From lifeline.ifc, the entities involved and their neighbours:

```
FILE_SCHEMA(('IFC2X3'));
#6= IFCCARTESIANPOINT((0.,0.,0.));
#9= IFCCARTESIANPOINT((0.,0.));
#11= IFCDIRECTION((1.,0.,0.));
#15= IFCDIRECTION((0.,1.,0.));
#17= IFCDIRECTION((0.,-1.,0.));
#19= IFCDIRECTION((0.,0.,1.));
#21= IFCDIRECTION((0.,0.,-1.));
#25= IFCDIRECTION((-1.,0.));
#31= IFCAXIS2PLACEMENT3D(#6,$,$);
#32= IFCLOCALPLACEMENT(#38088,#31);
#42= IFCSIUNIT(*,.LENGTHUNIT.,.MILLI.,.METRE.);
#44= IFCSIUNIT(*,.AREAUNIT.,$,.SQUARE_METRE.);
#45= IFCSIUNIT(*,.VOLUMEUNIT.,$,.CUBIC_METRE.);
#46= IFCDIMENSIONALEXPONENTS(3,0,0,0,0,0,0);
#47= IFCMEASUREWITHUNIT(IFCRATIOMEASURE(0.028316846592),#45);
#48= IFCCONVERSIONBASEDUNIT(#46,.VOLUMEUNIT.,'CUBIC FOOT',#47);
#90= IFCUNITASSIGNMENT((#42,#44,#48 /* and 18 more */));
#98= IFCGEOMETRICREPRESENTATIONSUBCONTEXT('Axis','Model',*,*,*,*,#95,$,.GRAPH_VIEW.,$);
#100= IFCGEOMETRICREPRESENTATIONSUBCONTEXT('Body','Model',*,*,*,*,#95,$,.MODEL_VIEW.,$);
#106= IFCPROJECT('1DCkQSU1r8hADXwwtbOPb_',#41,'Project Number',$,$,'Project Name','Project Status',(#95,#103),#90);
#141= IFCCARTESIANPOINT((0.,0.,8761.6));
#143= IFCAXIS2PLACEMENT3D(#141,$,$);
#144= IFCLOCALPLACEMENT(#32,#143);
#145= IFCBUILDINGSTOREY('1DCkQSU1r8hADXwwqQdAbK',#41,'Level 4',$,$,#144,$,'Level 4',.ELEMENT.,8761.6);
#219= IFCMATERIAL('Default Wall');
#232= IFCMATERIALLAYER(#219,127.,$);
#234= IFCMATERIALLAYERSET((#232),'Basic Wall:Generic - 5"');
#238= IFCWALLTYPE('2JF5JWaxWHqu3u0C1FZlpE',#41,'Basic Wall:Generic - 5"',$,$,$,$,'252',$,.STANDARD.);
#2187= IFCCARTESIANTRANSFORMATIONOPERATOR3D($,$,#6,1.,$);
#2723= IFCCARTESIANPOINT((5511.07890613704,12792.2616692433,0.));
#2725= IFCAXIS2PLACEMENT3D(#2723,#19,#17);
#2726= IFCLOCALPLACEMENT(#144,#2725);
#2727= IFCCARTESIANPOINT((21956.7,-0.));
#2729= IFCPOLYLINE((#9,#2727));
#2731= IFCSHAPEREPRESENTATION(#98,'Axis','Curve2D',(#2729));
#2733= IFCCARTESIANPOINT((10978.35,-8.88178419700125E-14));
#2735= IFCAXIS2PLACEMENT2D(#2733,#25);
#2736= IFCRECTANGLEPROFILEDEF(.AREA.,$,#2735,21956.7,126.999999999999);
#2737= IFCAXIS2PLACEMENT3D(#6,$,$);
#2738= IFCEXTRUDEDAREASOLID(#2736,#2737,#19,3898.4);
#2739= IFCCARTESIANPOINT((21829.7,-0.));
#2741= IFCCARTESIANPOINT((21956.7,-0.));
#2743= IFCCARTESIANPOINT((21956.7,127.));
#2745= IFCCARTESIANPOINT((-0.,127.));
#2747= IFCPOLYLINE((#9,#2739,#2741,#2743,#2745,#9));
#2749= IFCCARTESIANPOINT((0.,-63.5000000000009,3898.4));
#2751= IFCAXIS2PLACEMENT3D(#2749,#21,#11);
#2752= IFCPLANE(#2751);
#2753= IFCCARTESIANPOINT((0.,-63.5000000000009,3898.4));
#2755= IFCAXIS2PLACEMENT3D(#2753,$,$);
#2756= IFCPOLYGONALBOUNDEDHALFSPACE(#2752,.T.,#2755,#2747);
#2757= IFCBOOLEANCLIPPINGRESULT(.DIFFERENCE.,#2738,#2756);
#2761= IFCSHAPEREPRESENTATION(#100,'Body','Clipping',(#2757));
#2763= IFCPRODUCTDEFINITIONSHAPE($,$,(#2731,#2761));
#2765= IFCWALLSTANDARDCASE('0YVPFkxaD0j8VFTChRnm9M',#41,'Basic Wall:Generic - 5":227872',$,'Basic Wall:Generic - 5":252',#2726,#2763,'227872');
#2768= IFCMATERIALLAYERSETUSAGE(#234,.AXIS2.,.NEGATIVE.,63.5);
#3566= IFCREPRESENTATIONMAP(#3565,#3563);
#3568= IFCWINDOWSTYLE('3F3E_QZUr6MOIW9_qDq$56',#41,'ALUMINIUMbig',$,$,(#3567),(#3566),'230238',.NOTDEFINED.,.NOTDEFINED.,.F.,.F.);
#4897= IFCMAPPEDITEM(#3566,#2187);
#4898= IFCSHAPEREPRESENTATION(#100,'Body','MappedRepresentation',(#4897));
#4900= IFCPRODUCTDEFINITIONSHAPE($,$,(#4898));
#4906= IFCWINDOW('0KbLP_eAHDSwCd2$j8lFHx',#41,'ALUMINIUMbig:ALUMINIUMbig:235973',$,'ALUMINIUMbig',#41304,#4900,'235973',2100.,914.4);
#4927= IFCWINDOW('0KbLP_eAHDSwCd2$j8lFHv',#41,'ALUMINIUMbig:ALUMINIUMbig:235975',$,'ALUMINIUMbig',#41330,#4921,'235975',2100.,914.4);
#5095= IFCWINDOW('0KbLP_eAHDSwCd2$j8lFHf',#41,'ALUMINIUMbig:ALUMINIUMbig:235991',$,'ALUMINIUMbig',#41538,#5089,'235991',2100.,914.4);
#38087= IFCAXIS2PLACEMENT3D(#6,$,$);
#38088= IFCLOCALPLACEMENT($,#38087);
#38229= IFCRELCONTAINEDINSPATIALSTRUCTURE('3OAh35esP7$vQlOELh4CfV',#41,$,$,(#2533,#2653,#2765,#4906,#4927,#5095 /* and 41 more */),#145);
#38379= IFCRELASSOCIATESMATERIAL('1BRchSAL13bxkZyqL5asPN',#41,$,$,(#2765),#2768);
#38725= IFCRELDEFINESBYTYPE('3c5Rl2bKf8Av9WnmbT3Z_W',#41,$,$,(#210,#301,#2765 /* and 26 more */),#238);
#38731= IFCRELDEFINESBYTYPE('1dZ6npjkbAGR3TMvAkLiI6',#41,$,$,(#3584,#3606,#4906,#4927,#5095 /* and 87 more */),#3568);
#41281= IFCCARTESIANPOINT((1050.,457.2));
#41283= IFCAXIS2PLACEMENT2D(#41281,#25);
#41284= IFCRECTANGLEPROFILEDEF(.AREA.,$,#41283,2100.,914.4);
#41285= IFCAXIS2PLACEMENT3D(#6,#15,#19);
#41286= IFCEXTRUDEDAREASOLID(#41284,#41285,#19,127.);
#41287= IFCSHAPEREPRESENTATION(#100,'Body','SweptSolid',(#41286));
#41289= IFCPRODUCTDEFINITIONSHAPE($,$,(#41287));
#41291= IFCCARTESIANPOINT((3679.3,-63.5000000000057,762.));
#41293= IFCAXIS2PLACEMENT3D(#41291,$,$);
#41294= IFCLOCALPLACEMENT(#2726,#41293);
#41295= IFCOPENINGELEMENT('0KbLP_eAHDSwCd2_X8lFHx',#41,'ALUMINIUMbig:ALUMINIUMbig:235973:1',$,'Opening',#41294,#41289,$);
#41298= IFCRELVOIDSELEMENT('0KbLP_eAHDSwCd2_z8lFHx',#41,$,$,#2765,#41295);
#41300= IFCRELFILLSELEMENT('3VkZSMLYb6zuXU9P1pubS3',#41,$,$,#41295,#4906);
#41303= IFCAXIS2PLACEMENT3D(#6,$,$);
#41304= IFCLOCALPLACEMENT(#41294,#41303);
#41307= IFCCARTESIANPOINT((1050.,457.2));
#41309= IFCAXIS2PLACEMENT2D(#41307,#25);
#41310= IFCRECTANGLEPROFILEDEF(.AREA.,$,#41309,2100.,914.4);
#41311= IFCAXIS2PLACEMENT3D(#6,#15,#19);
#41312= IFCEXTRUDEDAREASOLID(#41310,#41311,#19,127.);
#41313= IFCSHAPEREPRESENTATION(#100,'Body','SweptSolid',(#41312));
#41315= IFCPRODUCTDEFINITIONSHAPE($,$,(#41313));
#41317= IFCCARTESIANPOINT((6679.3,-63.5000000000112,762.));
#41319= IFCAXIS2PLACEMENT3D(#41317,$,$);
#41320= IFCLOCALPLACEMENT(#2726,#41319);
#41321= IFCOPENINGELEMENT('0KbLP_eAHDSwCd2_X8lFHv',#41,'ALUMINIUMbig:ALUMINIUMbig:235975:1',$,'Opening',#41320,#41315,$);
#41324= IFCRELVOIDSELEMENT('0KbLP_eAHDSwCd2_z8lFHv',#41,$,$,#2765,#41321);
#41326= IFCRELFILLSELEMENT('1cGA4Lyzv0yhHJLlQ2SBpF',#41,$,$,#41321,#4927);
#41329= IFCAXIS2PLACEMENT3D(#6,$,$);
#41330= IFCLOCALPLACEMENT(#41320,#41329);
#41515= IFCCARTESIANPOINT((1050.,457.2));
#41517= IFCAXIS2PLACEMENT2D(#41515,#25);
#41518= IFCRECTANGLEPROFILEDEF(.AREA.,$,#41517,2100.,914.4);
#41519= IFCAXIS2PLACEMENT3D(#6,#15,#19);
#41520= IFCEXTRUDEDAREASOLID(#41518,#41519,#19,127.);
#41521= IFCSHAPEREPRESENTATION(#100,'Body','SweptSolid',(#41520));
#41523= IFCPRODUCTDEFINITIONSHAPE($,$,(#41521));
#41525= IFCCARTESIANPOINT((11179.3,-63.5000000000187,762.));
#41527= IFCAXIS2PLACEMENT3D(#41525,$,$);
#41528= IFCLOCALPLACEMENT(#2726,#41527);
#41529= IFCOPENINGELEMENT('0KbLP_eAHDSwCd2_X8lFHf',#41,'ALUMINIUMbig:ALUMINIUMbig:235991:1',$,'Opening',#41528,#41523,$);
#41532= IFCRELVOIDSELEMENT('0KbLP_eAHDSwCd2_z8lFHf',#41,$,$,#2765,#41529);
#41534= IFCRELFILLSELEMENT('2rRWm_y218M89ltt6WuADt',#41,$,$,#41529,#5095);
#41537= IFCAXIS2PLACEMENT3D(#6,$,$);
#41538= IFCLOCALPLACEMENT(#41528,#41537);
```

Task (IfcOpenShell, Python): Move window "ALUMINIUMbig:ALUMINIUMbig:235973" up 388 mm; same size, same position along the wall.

```python
import numpy as np
import ifcopenshell
import ifcopenshell.api.geometry
import ifcopenshell.util.placement
import ifcopenshell.util.unit

model = ifcopenshell.open("lifeline.ifc")
unit_scale = ifcopenshell.util.unit.calculate_unit_scale(model)

window = model.by_guid("0KbLP_eAHDSwCd2$j8lFHx")
opening = window.FillsVoids[0].RelatingOpeningElement
dz = 0.388 / unit_scale

shift = np.array([0.0, 0.0, dz])
# The window is placed relative to its opening, so it follows when the opening moves.
matrix = ifcopenshell.util.placement.get_local_placement(opening.ObjectPlacement)
matrix[:3, 3] += shift
ifcopenshell.api.geometry.edit_object_placement(
    model, product=opening, matrix=matrix, is_si=False, should_transform_children=True
)

print(f"moved by {dz * unit_scale:+.3f} m")

model.write("lifeline_rev.ifc")
```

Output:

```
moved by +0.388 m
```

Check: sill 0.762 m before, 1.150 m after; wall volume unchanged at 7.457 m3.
